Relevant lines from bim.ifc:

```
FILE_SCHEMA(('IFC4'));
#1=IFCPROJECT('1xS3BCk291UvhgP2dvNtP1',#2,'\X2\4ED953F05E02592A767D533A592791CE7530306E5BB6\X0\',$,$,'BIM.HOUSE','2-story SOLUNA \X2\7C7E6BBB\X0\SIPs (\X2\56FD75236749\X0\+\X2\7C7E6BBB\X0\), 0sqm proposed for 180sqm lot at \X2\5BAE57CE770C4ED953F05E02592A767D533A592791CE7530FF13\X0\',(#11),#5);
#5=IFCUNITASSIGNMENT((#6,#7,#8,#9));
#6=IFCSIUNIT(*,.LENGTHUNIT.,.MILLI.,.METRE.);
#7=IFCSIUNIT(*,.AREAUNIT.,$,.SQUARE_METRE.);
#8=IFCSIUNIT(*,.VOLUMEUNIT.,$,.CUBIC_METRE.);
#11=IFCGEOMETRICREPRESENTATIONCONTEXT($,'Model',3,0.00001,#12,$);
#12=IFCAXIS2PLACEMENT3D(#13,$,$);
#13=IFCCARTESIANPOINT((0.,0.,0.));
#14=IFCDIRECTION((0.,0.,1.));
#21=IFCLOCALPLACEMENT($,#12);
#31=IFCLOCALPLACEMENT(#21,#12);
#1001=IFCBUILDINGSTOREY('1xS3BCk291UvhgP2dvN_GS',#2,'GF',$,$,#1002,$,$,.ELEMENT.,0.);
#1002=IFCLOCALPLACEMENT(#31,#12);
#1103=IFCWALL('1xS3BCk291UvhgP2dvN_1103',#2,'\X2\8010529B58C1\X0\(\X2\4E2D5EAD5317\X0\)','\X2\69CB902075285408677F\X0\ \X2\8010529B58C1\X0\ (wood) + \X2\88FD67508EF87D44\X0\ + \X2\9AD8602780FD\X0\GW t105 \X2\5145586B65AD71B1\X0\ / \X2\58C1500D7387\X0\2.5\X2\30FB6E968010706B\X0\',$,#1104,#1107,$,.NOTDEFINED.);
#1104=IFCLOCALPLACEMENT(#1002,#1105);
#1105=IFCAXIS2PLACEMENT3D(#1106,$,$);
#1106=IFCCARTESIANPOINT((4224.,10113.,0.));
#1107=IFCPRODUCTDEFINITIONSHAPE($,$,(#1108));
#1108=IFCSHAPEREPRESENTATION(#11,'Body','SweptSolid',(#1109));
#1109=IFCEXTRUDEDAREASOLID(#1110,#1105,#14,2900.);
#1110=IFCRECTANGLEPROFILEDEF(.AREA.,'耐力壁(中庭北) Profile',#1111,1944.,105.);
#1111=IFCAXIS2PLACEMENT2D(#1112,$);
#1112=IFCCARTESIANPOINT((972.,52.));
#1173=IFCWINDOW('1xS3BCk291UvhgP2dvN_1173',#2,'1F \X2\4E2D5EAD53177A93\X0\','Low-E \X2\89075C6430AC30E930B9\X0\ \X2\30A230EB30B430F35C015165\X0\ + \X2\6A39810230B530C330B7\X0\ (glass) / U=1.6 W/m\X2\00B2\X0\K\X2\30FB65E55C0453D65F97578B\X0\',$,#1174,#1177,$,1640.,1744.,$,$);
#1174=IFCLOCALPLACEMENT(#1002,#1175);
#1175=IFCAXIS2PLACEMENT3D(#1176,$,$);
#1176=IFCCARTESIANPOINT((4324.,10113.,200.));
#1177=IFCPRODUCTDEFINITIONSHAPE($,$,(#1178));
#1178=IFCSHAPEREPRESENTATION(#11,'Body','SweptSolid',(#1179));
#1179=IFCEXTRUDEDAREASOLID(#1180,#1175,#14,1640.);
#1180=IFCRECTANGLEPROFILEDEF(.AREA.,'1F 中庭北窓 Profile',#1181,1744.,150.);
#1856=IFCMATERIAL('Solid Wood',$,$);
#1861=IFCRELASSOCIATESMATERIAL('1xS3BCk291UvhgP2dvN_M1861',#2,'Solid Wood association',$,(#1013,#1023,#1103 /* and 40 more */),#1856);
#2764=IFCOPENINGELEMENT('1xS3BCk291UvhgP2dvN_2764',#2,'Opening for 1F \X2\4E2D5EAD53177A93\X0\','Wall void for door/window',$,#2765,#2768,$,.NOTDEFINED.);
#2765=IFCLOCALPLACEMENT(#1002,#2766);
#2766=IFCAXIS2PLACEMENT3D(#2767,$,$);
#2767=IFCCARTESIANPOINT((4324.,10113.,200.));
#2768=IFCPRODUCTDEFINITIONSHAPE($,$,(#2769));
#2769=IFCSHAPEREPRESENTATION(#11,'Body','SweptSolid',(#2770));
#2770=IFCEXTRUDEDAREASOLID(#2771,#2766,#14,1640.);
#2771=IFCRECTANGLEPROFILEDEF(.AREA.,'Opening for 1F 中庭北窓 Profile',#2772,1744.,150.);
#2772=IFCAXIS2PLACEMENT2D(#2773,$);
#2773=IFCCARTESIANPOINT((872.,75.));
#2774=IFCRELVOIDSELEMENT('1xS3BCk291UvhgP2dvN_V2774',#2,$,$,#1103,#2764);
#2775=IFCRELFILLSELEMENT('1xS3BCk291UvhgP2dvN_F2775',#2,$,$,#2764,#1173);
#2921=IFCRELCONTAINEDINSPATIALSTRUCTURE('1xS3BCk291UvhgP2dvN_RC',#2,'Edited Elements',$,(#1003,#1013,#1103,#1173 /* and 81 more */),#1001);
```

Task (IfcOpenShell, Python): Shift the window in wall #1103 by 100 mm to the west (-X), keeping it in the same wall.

```python
import ifcopenshell
import ifcopenshell.api.geometry
import ifcopenshell.util.placement
import ifcopenshell.util.unit

model = ifcopenshell.open("bim.ifc")
unit_scale = ifcopenshell.util.unit.calculate_unit_scale(model)

window = model.by_guid("1xS3BCk291UvhgP2dvN_1173")
opening = window.FillsVoids[0].RelatingOpeningElement
wall = opening.VoidsElements[0].RelatingBuildingElement

wall_matrix = ifcopenshell.util.placement.get_local_placement(wall.ObjectPlacement)
shift = wall_matrix[:3, 0] * -0.1 / unit_scale
before = ifcopenshell.util.placement.get_local_placement(window.ObjectPlacement)[:3, 3].copy()

# The window is not placed relative to its opening, so move both.
for product in (opening, window):
    matrix = ifcopenshell.util.placement.get_local_placement(product.ObjectPlacement)
    matrix[:3, 3] += shift
    ifcopenshell.api.geometry.edit_object_placement(model, product=product, matrix=matrix, is_si=False)

after = ifcopenshell.util.placement.get_local_placement(window.ObjectPlacement)[:3, 3]
print("window moved by", (after - before).round(3) + 0.0)

model.write("bim_v2.ifc")
```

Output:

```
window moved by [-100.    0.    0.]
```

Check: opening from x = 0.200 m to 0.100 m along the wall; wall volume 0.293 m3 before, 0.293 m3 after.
